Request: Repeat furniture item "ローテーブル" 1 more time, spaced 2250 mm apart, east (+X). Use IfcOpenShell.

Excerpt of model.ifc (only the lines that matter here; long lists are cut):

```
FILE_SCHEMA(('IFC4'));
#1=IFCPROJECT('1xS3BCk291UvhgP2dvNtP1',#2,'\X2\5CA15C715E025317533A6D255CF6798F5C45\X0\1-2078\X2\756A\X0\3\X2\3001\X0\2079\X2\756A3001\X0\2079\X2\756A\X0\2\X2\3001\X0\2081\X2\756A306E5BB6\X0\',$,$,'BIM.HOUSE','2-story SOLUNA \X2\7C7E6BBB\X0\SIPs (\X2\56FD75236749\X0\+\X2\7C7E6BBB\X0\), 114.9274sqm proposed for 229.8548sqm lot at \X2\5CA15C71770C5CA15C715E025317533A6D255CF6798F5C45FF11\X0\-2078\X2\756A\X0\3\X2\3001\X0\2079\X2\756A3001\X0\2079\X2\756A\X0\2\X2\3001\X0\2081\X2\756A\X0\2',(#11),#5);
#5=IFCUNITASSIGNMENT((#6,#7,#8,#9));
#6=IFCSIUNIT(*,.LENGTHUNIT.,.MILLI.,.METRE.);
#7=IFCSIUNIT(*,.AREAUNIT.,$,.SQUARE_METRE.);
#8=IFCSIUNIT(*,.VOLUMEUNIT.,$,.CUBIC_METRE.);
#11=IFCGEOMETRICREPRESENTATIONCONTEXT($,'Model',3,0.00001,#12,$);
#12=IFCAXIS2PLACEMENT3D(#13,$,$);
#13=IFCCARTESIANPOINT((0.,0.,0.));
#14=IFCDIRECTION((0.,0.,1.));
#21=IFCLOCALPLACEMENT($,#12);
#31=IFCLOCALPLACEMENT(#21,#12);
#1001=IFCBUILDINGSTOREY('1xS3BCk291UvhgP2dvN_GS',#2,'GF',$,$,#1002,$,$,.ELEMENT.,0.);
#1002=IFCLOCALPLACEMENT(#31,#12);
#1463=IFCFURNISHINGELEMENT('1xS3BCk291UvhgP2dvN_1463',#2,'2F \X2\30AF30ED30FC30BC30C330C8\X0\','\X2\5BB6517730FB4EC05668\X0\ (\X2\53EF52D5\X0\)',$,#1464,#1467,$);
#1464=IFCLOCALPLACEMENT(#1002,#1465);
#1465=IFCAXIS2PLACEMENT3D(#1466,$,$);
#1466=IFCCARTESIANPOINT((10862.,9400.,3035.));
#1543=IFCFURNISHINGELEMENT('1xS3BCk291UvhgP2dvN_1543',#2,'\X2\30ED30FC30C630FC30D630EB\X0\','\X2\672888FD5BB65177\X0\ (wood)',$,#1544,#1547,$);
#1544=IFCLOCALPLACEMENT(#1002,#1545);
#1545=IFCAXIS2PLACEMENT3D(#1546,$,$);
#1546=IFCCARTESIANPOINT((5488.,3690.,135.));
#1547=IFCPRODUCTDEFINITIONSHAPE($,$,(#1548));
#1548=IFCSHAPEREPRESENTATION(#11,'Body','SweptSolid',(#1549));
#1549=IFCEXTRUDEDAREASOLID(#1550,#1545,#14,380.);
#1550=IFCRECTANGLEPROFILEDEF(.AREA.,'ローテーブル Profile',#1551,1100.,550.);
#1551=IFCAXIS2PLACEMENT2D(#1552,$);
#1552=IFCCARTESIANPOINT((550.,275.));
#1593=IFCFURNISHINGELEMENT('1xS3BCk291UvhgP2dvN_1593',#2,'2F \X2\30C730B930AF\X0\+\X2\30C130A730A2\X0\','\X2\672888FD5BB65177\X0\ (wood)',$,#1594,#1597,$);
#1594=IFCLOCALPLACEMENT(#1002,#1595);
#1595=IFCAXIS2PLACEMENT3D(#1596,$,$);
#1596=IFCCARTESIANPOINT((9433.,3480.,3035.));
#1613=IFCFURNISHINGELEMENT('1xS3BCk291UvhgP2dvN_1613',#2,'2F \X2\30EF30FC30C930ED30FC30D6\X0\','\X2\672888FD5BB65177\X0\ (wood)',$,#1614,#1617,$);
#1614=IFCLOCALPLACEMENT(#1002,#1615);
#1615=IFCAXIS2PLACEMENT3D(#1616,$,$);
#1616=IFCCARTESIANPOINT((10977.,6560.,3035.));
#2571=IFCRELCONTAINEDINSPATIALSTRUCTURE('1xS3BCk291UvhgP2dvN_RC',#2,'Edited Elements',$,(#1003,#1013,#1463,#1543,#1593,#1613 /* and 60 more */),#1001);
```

```python
import numpy as np
import ifcopenshell
import ifcopenshell.api.geometry
import ifcopenshell.api.root
import ifcopenshell.util.element
import ifcopenshell.util.placement

model = ifcopenshell.open("model.ifc")


def reuse_history(source, copy):
    """copy_class also copies each property set's owner history, people and application; keep the originals."""
    for rel in copy.IsDefinedBy:
        if rel.is_a("IfcRelDefinesByProperties") and (history := rel.RelatingPropertyDefinition.OwnerHistory):
            rel.RelatingPropertyDefinition.OwnerHistory = source.OwnerHistory
            ifcopenshell.util.element.remove_deep2(model, history)


source = model.by_id(1543)
base = ifcopenshell.util.placement.get_local_placement(source.ObjectPlacement)
step = np.array([1.0, 0.0, 0.0]) * 2250.0

for i in range(1, 2):
    copy = ifcopenshell.api.root.copy_class(model, product=source)
    copy.Representation = ifcopenshell.util.element.copy_deep(
        model, source.Representation, exclude=["IfcGeometricRepresentationContext", "IfcRepresentationMap"]
    )
    reuse_history(source, copy)
    matrix = base.copy()
    matrix[:3, 3] += i * step
    print("added at", matrix[:3, 3].round(3) + 0.0)
    ifcopenshell.api.geometry.edit_object_placement(model, product=copy, matrix=matrix, is_si=False)

model.write("model_v2.ifc")
```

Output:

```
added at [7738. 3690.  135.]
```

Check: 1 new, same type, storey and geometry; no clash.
